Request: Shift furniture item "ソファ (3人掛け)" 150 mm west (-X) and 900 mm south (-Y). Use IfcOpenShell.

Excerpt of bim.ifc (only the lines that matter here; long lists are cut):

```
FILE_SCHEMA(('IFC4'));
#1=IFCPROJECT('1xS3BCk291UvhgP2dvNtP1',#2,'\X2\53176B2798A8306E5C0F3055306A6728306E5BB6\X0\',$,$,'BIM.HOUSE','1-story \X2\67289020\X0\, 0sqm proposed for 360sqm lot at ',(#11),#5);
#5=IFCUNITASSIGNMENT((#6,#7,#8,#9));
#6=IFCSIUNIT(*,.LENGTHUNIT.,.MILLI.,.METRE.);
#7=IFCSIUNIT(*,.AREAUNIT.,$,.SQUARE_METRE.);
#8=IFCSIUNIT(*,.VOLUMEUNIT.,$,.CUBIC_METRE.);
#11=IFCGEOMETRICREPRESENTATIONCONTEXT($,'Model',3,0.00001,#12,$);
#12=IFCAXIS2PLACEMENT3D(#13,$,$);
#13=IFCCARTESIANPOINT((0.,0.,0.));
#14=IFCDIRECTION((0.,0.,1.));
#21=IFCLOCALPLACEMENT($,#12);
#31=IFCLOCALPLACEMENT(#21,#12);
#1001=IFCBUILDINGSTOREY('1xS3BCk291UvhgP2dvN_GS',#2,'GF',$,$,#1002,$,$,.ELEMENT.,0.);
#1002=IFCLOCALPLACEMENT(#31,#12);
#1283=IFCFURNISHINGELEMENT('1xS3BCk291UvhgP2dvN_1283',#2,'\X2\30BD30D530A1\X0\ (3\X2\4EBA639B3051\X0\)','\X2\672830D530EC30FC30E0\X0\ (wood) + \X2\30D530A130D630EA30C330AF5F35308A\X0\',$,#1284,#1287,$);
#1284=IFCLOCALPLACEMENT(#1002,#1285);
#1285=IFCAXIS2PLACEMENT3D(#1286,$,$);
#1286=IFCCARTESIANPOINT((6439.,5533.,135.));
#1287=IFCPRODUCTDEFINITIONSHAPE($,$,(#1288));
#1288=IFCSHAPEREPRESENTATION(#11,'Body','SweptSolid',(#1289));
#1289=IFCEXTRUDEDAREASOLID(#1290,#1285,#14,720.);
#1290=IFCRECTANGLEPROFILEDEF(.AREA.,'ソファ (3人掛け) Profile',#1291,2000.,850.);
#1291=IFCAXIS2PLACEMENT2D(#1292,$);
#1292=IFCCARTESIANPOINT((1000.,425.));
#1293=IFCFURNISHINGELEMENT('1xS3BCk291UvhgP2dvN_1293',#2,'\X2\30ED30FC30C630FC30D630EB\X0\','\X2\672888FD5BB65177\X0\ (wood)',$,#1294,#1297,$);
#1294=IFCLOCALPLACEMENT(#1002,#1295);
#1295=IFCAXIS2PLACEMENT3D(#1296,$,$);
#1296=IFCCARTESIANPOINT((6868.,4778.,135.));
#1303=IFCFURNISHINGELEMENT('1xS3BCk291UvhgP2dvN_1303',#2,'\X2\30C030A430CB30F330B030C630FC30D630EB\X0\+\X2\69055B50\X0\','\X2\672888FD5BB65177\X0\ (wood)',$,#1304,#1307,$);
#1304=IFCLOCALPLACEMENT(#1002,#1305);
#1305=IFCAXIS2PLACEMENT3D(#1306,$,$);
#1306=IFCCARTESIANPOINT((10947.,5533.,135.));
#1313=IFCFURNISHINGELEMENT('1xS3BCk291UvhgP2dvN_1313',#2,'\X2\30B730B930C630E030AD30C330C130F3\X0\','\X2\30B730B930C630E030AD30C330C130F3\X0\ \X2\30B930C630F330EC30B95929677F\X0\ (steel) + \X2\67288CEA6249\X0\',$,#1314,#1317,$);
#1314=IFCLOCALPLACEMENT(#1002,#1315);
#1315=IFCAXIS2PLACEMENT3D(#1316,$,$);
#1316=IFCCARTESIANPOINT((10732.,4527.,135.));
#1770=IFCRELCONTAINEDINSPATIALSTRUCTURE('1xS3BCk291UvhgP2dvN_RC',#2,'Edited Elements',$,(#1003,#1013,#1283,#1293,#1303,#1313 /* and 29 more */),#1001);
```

```python
import ifcopenshell
import ifcopenshell.api.geometry
import ifcopenshell.util.placement

model = ifcopenshell.open("bim.ifc")

item = model.by_guid("1xS3BCk291UvhgP2dvN_1283")
matrix = ifcopenshell.util.placement.get_local_placement(item.ObjectPlacement)
matrix[0, 3] -= 150.0
matrix[1, 3] -= 900.0
ifcopenshell.api.geometry.edit_object_placement(model, product=item, matrix=matrix, is_si=False)

print(ifcopenshell.util.placement.get_local_placement(item.ObjectPlacement).round(3) + 0.0)

model.write("bim_edited.ifc")
```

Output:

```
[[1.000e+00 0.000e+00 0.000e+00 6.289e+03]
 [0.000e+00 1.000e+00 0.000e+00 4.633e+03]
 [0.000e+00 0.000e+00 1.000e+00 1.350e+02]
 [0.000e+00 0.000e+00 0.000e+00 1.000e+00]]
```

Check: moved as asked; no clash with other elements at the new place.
